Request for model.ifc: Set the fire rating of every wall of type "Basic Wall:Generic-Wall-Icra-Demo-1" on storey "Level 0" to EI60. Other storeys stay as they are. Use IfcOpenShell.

First a look at what the model holds.

```python
import ifcopenshell
import ifcopenshell.util.element

model = ifcopenshell.open("model.ifc")
print(model.schema)
storey = next(s for s in model.by_type("IfcBuildingStorey") if s.Name == "Level 0")
walls = [e for e in ifcopenshell.util.element.get_decomposition(storey) if e.is_a("IfcWall")]
seen = {}
for e in walls:
    element_type = ifcopenshell.util.element.get_type(e)
    key = (element_type.Name if element_type != e and element_type else None, ifcopenshell.util.element.get_pset(e, "Pset_WallCommon", "FireRating"))
    seen[key] = seen.get(key, 0) + 1
for (name, value), count in sorted(seen.items(), key=str):
    print(count, "x", name, "|", value)
```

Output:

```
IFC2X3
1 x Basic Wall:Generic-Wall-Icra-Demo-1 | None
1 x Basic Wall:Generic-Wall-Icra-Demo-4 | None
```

```python
import ifcopenshell
import ifcopenshell.api.pset
import ifcopenshell.util.element

model = ifcopenshell.open("model.ifc")

storey = next(s for s in model.by_type("IfcBuildingStorey") if s.Name == "Level 0")
walls = [e for e in ifcopenshell.util.element.get_decomposition(storey) if e.is_a("IfcWall")]

count = 0
for e in walls:
    element_type = ifcopenshell.util.element.get_type(e)
    if element_type in (None, e) or element_type.Name != "Basic Wall:Generic-Wall-Icra-Demo-1":
        continue
    # add_pset returns the element's existing set when there is one.
    pset = ifcopenshell.api.pset.add_pset(model, product=e, name="Pset_WallCommon")
    ifcopenshell.api.pset.edit_pset(model, pset=pset, properties={"FireRating": "EI60"})
    count += 1

print(count, "walls updated")

model.write("model-out.ifc")
```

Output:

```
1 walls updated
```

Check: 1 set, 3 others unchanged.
